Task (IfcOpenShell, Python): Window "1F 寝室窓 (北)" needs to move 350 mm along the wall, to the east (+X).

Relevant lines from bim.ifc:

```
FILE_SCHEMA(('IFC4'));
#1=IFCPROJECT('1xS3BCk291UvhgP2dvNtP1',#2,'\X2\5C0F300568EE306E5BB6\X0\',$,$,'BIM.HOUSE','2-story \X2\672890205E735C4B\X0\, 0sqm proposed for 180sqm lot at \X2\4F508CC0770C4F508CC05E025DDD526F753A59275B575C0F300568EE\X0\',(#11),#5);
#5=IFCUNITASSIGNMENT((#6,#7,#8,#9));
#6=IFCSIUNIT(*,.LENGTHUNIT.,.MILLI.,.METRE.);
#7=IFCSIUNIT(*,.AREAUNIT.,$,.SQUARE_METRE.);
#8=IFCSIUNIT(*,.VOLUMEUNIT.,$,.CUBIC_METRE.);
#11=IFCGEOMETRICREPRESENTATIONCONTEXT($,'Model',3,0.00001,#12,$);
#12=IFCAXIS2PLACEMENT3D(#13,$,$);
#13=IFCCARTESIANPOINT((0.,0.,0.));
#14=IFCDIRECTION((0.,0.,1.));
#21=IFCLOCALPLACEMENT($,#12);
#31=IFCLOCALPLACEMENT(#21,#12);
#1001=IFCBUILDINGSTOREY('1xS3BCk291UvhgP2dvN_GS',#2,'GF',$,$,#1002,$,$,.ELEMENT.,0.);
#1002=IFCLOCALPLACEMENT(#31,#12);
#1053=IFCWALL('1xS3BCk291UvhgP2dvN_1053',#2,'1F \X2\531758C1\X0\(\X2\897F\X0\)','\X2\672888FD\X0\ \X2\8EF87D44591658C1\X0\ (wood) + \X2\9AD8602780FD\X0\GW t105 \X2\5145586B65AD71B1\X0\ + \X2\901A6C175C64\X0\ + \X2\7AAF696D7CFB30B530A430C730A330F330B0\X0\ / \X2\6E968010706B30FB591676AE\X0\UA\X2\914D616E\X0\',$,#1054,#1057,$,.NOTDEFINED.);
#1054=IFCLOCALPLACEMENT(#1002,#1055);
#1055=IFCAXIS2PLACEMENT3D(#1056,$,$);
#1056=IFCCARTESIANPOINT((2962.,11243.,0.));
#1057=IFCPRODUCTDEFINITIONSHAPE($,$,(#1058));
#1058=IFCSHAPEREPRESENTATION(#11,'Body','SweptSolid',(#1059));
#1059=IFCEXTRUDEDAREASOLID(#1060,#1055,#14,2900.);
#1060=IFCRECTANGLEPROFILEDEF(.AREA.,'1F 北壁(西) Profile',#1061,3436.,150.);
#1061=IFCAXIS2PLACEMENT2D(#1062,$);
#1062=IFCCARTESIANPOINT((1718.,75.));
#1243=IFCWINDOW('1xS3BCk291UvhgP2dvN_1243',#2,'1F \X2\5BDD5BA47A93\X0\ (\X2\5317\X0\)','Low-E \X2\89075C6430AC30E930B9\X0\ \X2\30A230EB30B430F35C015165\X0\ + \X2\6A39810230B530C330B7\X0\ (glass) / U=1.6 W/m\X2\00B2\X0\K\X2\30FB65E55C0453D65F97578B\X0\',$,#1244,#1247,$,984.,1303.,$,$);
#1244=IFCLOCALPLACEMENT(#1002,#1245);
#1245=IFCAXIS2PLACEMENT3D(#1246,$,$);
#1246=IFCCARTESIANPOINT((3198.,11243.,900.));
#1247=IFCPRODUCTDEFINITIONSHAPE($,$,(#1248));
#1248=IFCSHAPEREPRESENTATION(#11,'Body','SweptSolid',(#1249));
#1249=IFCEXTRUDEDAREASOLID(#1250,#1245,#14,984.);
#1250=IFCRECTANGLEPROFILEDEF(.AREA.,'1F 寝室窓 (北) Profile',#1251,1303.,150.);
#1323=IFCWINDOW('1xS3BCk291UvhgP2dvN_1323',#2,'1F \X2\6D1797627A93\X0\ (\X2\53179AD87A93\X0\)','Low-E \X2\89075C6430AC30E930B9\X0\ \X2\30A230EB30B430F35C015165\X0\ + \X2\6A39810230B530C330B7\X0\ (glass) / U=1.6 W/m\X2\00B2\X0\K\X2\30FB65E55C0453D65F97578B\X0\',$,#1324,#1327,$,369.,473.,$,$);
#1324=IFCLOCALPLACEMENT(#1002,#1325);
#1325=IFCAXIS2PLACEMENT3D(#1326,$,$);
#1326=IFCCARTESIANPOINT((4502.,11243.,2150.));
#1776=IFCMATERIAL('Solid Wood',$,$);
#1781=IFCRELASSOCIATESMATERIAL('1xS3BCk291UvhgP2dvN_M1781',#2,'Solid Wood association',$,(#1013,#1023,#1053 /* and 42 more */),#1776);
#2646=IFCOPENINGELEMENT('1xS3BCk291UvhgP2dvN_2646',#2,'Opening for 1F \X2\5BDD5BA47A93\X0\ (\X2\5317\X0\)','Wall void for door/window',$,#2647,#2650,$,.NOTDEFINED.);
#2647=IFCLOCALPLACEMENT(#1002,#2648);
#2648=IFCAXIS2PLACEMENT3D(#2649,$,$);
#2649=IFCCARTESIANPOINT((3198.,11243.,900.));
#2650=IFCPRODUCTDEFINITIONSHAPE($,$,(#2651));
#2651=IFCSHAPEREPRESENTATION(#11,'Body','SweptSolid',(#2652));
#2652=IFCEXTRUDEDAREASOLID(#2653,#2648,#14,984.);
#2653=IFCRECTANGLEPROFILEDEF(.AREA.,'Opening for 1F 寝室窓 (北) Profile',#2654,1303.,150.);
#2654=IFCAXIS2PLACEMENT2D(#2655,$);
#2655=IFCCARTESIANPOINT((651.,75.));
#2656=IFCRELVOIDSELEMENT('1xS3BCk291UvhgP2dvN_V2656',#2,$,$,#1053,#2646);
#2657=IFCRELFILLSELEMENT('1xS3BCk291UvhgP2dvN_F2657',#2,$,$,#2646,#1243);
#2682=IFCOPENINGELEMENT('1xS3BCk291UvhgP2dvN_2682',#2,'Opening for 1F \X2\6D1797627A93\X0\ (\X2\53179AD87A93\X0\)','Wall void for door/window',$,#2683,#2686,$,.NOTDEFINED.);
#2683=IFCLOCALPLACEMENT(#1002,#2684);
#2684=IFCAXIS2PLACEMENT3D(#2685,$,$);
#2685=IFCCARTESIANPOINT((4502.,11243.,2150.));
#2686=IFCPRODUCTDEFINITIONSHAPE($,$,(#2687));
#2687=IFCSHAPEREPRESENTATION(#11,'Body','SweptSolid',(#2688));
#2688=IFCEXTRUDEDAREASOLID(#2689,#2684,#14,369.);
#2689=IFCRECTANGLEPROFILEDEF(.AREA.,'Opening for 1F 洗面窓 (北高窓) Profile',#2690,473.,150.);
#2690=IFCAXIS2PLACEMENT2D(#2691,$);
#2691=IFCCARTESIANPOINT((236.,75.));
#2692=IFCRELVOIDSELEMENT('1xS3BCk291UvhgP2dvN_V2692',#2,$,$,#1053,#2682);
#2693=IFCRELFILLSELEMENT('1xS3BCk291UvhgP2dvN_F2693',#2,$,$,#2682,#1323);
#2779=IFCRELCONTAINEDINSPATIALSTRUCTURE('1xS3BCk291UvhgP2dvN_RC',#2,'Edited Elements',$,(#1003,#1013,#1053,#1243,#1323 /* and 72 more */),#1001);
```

```python
import ifcopenshell
import ifcopenshell.api.geometry
import ifcopenshell.util.placement

model = ifcopenshell.open("bim.ifc")

window = model.by_id(1243)
opening = window.FillsVoids[0].RelatingOpeningElement
wall = opening.VoidsElements[0].RelatingBuildingElement

wall_matrix = ifcopenshell.util.placement.get_local_placement(wall.ObjectPlacement)
shift = wall_matrix[:3, 0] * 350.0
before = ifcopenshell.util.placement.get_local_placement(window.ObjectPlacement)[:3, 3].copy()

# The window is not placed relative to its opening, so move both.
for product in (opening, window):
    matrix = ifcopenshell.util.placement.get_local_placement(product.ObjectPlacement)
    matrix[:3, 3] += shift
    ifcopenshell.api.geometry.edit_object_placement(model, product=product, matrix=matrix, is_si=False)

after = ifcopenshell.util.placement.get_local_placement(window.ObjectPlacement)[:3, 3]
print("window moved by", (after - before).round(3) + 0.0)

model.write("bim_v2.ifc")
```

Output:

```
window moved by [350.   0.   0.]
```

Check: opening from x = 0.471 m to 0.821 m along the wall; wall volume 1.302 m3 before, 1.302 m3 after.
